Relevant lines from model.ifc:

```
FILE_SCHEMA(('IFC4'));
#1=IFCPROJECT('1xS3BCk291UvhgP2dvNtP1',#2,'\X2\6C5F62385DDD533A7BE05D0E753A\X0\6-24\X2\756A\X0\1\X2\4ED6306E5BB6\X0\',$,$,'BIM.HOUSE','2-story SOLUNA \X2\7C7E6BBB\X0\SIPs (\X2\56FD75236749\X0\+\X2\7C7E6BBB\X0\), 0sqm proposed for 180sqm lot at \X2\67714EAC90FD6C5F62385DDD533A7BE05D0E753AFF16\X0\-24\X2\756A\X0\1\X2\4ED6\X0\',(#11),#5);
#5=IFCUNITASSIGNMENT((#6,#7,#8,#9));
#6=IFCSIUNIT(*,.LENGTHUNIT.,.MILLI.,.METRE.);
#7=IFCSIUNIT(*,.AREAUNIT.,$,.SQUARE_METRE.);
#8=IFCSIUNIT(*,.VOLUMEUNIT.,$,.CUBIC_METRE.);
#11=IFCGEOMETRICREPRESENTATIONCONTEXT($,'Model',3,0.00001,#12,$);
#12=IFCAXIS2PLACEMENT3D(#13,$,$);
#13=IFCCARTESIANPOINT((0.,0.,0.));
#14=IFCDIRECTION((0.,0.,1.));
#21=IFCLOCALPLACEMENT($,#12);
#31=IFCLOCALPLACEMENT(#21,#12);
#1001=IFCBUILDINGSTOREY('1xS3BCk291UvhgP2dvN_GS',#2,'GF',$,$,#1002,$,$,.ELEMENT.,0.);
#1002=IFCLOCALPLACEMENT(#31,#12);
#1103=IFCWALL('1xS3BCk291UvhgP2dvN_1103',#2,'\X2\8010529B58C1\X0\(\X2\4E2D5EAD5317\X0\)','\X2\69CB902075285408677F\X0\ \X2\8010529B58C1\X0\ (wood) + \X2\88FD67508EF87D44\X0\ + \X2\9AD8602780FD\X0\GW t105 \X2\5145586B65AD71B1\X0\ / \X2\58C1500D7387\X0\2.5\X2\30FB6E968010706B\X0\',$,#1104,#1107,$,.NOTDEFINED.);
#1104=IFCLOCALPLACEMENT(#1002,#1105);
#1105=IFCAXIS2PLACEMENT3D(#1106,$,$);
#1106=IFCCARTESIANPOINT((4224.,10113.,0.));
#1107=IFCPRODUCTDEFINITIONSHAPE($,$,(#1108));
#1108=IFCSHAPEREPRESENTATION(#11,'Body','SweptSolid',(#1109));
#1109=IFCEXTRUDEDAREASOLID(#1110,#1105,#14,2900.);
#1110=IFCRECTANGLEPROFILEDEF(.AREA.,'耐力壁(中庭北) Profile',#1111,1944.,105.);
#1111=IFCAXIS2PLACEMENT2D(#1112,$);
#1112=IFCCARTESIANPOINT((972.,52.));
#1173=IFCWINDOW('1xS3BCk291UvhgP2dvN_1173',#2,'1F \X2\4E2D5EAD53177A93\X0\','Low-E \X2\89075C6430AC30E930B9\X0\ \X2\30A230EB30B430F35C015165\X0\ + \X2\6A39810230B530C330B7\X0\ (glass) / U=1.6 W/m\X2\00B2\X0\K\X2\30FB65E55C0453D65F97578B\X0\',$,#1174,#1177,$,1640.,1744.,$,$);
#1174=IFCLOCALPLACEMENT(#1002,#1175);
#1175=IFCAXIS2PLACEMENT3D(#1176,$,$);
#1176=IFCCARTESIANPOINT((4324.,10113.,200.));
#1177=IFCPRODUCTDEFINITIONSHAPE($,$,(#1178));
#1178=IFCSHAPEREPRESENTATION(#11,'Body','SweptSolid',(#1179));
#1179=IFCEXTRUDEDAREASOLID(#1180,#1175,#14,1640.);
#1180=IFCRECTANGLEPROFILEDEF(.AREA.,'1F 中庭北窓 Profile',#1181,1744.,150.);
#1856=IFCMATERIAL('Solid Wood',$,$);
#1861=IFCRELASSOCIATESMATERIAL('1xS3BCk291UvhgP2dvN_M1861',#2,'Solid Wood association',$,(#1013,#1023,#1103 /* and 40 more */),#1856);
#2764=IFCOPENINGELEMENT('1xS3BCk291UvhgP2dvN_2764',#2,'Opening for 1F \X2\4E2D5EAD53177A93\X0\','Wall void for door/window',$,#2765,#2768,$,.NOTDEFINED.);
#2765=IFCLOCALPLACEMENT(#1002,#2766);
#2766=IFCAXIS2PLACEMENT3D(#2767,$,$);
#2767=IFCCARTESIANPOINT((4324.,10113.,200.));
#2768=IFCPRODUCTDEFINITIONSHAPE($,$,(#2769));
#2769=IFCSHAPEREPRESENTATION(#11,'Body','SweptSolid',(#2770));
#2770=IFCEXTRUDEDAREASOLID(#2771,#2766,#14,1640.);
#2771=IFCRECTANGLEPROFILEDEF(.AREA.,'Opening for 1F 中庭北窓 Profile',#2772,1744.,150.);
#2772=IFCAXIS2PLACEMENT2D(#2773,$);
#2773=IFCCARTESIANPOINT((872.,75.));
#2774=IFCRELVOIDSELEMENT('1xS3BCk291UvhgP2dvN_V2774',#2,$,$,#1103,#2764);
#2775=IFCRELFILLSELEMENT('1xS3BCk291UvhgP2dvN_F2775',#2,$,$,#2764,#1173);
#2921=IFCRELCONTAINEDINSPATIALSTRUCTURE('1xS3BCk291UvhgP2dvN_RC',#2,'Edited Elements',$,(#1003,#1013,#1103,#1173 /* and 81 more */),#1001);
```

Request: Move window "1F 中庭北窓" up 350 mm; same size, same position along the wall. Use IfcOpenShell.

```python
import numpy as np
import ifcopenshell
import ifcopenshell.api.geometry
import ifcopenshell.util.placement
import ifcopenshell.util.unit

model = ifcopenshell.open("model.ifc")
unit_scale = ifcopenshell.util.unit.calculate_unit_scale(model)

window = model.by_guid("1xS3BCk291UvhgP2dvN_1173")
opening = window.FillsVoids[0].RelatingOpeningElement
dz = 350.0

shift = np.array([0.0, 0.0, dz])
# The window is not placed relative to its opening, so move both.
for product in (opening, window):
    matrix = ifcopenshell.util.placement.get_local_placement(product.ObjectPlacement)
    matrix[:3, 3] += shift
    ifcopenshell.api.geometry.edit_object_placement(model, product=product, matrix=matrix, is_si=False)

print(f"moved by {dz * unit_scale:+.3f} m")

model.write("model_v2.ifc")
```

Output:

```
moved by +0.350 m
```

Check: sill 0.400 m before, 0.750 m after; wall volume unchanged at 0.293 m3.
